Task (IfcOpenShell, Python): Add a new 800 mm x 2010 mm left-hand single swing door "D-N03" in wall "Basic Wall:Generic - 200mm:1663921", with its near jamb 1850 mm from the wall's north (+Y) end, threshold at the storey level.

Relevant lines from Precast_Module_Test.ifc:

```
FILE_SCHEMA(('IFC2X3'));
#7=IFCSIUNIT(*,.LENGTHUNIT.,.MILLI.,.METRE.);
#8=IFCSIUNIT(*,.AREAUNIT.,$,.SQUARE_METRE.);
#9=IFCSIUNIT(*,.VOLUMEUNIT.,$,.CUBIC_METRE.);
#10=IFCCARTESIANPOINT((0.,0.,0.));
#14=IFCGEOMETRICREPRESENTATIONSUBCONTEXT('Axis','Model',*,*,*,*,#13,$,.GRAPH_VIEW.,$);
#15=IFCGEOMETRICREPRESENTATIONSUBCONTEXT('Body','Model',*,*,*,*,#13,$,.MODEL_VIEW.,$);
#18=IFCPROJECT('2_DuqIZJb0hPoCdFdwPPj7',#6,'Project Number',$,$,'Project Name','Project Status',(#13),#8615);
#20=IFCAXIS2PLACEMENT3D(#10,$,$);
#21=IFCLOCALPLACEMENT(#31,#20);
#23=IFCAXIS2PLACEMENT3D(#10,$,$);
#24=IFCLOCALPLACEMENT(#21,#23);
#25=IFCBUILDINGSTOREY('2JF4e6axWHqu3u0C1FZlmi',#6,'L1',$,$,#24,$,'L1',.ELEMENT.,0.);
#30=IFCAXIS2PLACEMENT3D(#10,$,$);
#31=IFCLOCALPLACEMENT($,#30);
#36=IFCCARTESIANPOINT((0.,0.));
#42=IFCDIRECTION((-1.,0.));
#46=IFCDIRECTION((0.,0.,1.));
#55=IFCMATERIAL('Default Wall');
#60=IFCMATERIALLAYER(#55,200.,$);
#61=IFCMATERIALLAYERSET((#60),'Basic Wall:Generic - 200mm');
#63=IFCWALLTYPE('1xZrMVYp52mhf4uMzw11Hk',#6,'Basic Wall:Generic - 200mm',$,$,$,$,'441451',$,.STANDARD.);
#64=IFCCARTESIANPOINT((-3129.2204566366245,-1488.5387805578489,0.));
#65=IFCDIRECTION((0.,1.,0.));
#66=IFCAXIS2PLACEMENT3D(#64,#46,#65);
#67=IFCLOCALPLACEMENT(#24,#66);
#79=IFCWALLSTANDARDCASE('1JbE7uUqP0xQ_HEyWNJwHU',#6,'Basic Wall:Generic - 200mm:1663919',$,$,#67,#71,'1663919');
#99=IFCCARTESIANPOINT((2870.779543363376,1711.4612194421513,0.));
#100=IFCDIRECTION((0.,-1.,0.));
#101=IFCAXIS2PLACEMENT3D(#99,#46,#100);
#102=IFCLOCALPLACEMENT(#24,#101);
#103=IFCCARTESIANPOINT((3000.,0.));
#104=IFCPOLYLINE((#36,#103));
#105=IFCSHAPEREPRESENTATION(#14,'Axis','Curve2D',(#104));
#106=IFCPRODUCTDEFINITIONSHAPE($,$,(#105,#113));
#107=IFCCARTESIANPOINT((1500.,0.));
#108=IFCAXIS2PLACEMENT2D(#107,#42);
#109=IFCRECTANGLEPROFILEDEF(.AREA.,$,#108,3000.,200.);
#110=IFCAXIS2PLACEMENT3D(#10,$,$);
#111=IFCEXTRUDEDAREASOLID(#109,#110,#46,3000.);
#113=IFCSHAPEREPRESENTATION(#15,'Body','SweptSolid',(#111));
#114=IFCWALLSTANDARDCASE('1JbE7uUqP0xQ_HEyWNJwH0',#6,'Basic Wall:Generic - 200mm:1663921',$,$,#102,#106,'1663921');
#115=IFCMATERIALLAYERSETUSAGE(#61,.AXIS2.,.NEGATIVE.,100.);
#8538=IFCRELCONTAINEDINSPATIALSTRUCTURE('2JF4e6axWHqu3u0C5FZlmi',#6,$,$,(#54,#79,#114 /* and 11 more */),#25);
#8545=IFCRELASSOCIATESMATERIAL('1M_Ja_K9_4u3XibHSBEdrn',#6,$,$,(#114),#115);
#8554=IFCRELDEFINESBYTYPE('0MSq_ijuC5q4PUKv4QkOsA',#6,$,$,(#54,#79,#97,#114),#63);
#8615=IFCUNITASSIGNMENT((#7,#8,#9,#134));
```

```python
import numpy as np
import ifcopenshell
import ifcopenshell.api.feature
import ifcopenshell.api.geometry
import ifcopenshell.api.root
import ifcopenshell.api.spatial
import ifcopenshell.api.type
import ifcopenshell.geom
import ifcopenshell.util.element
import ifcopenshell.util.placement
import ifcopenshell.util.representation
import ifcopenshell.util.shape
import ifcopenshell.util.unit

model = ifcopenshell.open("Precast_Module_Test.ifc")
unit_scale = ifcopenshell.util.unit.calculate_unit_scale(model)
settings = ifcopenshell.geom.settings()


def volume(element):
    """Net volume in cubic metres, openings subtracted."""
    shape = ifcopenshell.geom.create_shape(settings, element)
    return ifcopenshell.util.shape.get_volume(shape.geometry)


wall = model.by_id(114)
storey = ifcopenshell.util.element.get_container(wall, ifc_class="IfcBuildingStorey")
context = ifcopenshell.util.representation.get_context(model, "Model", "Body", "MODEL_VIEW")
before = volume(wall)

width, height, from_end, sill = 0.8, 2.01, 1.85, 0.0  # metres

# The wall runs along its own X axis, and the end named is its -X end.
wall_shape = ifcopenshell.geom.create_shape(settings, wall)
x, y, z = ifcopenshell.util.shape.get_vertices(wall_shape.geometry).T
start = x.min() + from_end
face, thickness = float(y.min()), float(y.max() - y.min())
wall_matrix = ifcopenshell.util.placement.get_local_placement(wall.ObjectPlacement)
level = ifcopenshell.util.placement.get_local_placement(storey.ObjectPlacement)[2, 3]


def in_wall(x, y):
    """Placement at x, y metres in the wall's axes, at sill height."""
    matrix = wall_matrix.copy()
    matrix[:, 3] = wall_matrix @ np.array([x / unit_scale, y / unit_scale, 0.0, 1.0])
    matrix[2, 3] = level + sill / unit_scale
    return matrix


# Opening: a box that overshoots both wall faces by 50 mm.
opening = ifcopenshell.api.root.create_entity(model, ifc_class="IfcOpeningElement")
box = ifcopenshell.api.geometry.add_wall_representation(
    model, context=context, length=width, height=height, thickness=thickness + 0.1
)
ifcopenshell.api.geometry.assign_representation(model, product=opening, representation=box)
ifcopenshell.api.geometry.edit_object_placement(model, product=opening, matrix=in_wall(start, face - 0.05), is_si=False)
ifcopenshell.api.feature.add_feature(model, feature=opening, element=wall)

door = ifcopenshell.api.root.create_entity(model, ifc_class="IfcDoor", name="D-N03")
door.OverallWidth, door.OverallHeight = width / unit_scale, height / unit_scale
body = ifcopenshell.api.geometry.add_door_representation(
    model,
    context=context,
    overall_width=door.OverallWidth,
    overall_height=door.OverallHeight,
    operation_type="SINGLE_SWING_LEFT",
    lining_properties={"LiningDepth": thickness / unit_scale, "ThresholdDepth": thickness / unit_scale},
)
ifcopenshell.api.geometry.assign_representation(model, product=door, representation=body)
ifcopenshell.api.spatial.assign_container(model, products=[door], relating_structure=storey)
fills = ifcopenshell.api.feature.add_filling(model, opening=opening, element=door)
fills.OwnerHistory = door.OwnerHistory  # required in IFC2X3

# IFC2X3 keeps the operation on the door style.
style = ifcopenshell.api.root.create_entity(model, ifc_class="IfcDoorStyle", name="D-N03")
style.OperationType, style.ConstructionType = "SINGLE_SWING_LEFT", "NOTDEFINED"
style.ParameterTakesPrecedence = style.Sizeable = False
ifcopenshell.api.type.assign_type(model, related_objects=[door], relating_type=style)

# The lining spans the wall, so the door starts at the wall face.
ifcopenshell.api.geometry.edit_object_placement(model, product=door, matrix=in_wall(start, face), is_si=False)

after = volume(wall)

print(f"wall volume {before:.3f} -> {after:.3f} m3")

model.write("Precast_Module_Test_rev.ifc")
```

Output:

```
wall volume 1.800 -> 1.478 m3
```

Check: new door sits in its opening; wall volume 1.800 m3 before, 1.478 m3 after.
